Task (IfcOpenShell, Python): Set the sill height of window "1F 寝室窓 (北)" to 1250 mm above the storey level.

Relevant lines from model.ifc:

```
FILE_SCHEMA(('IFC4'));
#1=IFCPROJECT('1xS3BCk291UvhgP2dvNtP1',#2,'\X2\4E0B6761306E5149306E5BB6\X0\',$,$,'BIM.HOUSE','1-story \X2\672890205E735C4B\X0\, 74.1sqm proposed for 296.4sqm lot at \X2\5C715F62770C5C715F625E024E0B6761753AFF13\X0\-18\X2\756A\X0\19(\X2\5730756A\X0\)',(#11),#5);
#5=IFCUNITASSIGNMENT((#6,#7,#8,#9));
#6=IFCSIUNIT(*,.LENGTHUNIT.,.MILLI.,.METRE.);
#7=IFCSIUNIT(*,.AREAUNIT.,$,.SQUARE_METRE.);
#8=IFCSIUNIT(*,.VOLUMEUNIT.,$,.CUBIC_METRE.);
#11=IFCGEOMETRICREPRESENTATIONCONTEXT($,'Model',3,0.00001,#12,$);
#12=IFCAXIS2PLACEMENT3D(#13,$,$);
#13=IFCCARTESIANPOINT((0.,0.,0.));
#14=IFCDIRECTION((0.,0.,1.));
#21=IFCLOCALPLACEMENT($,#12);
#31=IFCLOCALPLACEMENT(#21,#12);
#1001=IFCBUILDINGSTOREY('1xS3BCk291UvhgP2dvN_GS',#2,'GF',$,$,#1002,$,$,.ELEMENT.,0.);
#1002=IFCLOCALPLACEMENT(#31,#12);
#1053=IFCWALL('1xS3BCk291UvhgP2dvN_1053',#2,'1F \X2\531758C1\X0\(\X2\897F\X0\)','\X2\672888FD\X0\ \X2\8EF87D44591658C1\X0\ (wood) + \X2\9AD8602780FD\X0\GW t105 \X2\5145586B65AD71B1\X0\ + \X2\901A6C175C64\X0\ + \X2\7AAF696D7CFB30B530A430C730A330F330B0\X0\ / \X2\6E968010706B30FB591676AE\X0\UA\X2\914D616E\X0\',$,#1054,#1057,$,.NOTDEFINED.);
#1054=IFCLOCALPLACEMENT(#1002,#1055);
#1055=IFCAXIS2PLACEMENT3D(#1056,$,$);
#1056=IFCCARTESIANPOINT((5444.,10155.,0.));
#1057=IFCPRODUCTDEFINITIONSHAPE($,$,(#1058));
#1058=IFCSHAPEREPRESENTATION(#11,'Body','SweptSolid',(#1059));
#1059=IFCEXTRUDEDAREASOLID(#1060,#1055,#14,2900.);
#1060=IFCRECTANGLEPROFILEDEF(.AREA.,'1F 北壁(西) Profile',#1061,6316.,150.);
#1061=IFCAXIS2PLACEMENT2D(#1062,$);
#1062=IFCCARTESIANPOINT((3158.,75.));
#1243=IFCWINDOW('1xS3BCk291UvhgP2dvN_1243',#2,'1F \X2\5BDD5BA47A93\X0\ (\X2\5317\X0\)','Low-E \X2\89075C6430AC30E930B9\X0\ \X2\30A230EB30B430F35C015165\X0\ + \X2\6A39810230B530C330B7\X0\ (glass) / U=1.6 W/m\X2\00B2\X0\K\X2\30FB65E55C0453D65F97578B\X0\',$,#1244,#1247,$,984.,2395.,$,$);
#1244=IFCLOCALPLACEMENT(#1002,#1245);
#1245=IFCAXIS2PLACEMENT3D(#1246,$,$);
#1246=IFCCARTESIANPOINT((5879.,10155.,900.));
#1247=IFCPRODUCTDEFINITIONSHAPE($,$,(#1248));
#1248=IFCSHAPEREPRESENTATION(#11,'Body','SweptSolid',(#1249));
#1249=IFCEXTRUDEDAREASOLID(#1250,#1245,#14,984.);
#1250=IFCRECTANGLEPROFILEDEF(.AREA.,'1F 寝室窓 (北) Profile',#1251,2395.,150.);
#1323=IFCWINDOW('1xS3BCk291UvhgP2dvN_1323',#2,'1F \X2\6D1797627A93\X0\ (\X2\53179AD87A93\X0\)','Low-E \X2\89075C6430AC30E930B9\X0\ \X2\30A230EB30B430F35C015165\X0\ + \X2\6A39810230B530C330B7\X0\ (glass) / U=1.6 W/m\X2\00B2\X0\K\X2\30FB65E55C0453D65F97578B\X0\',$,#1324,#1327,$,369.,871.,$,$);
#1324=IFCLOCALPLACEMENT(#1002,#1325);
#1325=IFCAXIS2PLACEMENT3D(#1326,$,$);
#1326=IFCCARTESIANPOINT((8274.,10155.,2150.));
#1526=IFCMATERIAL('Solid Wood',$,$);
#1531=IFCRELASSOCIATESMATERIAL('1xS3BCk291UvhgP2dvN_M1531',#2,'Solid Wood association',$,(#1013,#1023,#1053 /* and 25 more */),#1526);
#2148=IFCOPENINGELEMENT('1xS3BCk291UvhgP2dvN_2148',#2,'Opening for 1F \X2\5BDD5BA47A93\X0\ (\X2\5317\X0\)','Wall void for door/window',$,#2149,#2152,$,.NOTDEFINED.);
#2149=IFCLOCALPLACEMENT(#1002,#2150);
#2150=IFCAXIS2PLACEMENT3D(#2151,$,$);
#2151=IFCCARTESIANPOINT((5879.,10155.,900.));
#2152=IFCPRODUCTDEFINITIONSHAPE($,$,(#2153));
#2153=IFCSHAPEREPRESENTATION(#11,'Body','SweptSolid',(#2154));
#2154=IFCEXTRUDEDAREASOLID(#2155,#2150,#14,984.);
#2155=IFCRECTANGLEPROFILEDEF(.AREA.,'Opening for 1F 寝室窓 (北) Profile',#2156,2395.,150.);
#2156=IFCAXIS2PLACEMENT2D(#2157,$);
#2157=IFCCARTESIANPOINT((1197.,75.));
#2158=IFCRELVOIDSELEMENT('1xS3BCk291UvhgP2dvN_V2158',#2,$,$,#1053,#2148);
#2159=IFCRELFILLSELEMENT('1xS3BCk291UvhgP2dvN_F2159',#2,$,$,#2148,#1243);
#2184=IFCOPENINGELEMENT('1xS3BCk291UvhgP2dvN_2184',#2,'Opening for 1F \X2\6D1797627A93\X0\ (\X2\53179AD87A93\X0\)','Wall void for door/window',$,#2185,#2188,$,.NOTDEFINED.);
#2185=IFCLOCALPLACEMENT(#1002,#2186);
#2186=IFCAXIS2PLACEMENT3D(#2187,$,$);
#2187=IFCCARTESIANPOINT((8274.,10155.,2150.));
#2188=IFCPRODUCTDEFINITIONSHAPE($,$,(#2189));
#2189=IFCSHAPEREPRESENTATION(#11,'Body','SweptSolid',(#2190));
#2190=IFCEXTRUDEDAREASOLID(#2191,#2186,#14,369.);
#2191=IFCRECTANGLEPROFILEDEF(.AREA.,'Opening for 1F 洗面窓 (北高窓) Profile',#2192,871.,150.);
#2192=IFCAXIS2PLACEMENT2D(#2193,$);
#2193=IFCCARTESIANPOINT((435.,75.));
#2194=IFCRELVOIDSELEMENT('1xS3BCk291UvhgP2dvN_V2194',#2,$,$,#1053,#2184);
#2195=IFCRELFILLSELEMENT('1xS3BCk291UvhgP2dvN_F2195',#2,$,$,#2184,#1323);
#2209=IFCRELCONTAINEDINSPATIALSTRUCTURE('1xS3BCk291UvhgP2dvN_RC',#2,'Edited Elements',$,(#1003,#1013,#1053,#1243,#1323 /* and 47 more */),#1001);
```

```python
import numpy as np
import ifcopenshell
import ifcopenshell.api.geometry
import ifcopenshell.geom
import ifcopenshell.util.element
import ifcopenshell.util.placement
import ifcopenshell.util.shape
import ifcopenshell.util.unit

model = ifcopenshell.open("model.ifc")
unit_scale = ifcopenshell.util.unit.calculate_unit_scale(model)

window = model.by_id(1243)
opening = window.FillsVoids[0].RelatingOpeningElement
storey = ifcopenshell.util.element.get_container(window, ifc_class="IfcBuildingStorey")
level = ifcopenshell.util.placement.get_local_placement(storey.ObjectPlacement)[2, 3]

# The opening's origin need not be at the sill, so measure its lowest point.
shape = ifcopenshell.geom.create_shape(ifcopenshell.geom.settings(), opening)
bottom = ifcopenshell.util.shape.get_shape_bottom_elevation(shape, shape.geometry) / unit_scale
dz = level + 1250.0 - bottom

shift = np.array([0.0, 0.0, dz])
# The window is not placed relative to its opening, so move both.
for product in (opening, window):
    matrix = ifcopenshell.util.placement.get_local_placement(product.ObjectPlacement)
    matrix[:3, 3] += shift
    ifcopenshell.api.geometry.edit_object_placement(model, product=product, matrix=matrix, is_si=False)

print(f"moved by {dz * unit_scale:+.3f} m")

model.write("model_edited.ifc")
```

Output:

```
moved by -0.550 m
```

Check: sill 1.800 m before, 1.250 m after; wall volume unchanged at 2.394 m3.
